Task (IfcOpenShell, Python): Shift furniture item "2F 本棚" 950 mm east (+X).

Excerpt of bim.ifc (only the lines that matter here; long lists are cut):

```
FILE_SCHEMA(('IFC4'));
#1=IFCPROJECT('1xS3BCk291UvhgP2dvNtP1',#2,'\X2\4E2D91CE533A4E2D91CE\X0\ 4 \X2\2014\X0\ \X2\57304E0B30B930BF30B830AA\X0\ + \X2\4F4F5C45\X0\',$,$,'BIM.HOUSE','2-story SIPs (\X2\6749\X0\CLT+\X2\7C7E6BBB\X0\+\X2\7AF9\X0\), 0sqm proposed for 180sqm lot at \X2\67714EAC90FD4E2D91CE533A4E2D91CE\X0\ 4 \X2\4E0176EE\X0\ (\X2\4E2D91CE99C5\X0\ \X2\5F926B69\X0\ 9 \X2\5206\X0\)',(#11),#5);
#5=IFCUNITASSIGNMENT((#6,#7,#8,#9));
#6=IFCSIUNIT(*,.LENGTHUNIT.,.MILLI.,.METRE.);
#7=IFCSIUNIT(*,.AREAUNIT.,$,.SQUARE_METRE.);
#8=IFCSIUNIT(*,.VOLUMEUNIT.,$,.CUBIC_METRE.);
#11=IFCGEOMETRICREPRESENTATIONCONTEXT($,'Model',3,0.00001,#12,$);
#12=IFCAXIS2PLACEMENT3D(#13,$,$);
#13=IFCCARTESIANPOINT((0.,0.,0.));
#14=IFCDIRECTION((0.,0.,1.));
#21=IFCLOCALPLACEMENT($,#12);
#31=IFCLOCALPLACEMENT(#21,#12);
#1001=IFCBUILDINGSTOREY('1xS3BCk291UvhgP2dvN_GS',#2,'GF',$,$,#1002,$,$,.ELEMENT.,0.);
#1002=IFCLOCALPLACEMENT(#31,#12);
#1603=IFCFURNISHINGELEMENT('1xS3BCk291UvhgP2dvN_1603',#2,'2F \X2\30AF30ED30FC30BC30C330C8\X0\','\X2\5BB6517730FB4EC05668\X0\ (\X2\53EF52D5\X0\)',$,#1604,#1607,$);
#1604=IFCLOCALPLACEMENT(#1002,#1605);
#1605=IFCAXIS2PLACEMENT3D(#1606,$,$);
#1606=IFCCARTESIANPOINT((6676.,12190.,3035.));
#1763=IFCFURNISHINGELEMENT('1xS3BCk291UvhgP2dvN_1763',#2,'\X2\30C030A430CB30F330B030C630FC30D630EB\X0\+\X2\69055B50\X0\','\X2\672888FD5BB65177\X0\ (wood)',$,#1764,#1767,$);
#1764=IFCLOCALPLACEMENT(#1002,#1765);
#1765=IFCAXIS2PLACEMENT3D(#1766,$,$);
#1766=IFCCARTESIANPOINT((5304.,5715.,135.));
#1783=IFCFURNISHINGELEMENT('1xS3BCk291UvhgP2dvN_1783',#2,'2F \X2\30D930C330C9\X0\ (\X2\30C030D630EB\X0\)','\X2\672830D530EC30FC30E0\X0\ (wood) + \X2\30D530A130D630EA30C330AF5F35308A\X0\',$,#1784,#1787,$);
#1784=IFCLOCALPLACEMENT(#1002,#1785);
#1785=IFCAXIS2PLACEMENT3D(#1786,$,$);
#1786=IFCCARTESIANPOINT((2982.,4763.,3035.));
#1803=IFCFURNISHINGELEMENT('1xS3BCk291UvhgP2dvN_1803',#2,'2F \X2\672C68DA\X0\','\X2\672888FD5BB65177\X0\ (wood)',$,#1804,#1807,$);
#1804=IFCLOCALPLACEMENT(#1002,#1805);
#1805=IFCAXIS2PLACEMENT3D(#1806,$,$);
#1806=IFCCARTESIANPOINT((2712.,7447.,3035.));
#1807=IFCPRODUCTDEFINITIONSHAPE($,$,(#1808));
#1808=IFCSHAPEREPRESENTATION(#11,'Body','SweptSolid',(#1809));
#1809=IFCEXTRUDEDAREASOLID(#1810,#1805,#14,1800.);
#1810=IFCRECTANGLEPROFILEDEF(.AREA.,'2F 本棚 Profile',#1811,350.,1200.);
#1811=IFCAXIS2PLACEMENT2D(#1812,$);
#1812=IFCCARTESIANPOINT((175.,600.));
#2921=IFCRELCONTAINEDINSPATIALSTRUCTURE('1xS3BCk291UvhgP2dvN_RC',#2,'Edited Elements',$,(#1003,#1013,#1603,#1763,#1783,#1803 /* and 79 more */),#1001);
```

```python
import ifcopenshell
import ifcopenshell.api.geometry
import ifcopenshell.util.placement

model = ifcopenshell.open("bim.ifc")

item = model.by_guid("1xS3BCk291UvhgP2dvN_1803")
matrix = ifcopenshell.util.placement.get_local_placement(item.ObjectPlacement)
matrix[0, 3] += 950.0
ifcopenshell.api.geometry.edit_object_placement(model, product=item, matrix=matrix, is_si=False)

print(ifcopenshell.util.placement.get_local_placement(item.ObjectPlacement).round(3) + 0.0)

model.write("bim_updated.ifc")
```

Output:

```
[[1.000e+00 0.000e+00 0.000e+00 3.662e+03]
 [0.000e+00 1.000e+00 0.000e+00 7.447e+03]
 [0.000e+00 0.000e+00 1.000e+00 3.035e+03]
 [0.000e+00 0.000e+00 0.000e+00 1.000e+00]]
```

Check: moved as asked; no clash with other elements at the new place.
